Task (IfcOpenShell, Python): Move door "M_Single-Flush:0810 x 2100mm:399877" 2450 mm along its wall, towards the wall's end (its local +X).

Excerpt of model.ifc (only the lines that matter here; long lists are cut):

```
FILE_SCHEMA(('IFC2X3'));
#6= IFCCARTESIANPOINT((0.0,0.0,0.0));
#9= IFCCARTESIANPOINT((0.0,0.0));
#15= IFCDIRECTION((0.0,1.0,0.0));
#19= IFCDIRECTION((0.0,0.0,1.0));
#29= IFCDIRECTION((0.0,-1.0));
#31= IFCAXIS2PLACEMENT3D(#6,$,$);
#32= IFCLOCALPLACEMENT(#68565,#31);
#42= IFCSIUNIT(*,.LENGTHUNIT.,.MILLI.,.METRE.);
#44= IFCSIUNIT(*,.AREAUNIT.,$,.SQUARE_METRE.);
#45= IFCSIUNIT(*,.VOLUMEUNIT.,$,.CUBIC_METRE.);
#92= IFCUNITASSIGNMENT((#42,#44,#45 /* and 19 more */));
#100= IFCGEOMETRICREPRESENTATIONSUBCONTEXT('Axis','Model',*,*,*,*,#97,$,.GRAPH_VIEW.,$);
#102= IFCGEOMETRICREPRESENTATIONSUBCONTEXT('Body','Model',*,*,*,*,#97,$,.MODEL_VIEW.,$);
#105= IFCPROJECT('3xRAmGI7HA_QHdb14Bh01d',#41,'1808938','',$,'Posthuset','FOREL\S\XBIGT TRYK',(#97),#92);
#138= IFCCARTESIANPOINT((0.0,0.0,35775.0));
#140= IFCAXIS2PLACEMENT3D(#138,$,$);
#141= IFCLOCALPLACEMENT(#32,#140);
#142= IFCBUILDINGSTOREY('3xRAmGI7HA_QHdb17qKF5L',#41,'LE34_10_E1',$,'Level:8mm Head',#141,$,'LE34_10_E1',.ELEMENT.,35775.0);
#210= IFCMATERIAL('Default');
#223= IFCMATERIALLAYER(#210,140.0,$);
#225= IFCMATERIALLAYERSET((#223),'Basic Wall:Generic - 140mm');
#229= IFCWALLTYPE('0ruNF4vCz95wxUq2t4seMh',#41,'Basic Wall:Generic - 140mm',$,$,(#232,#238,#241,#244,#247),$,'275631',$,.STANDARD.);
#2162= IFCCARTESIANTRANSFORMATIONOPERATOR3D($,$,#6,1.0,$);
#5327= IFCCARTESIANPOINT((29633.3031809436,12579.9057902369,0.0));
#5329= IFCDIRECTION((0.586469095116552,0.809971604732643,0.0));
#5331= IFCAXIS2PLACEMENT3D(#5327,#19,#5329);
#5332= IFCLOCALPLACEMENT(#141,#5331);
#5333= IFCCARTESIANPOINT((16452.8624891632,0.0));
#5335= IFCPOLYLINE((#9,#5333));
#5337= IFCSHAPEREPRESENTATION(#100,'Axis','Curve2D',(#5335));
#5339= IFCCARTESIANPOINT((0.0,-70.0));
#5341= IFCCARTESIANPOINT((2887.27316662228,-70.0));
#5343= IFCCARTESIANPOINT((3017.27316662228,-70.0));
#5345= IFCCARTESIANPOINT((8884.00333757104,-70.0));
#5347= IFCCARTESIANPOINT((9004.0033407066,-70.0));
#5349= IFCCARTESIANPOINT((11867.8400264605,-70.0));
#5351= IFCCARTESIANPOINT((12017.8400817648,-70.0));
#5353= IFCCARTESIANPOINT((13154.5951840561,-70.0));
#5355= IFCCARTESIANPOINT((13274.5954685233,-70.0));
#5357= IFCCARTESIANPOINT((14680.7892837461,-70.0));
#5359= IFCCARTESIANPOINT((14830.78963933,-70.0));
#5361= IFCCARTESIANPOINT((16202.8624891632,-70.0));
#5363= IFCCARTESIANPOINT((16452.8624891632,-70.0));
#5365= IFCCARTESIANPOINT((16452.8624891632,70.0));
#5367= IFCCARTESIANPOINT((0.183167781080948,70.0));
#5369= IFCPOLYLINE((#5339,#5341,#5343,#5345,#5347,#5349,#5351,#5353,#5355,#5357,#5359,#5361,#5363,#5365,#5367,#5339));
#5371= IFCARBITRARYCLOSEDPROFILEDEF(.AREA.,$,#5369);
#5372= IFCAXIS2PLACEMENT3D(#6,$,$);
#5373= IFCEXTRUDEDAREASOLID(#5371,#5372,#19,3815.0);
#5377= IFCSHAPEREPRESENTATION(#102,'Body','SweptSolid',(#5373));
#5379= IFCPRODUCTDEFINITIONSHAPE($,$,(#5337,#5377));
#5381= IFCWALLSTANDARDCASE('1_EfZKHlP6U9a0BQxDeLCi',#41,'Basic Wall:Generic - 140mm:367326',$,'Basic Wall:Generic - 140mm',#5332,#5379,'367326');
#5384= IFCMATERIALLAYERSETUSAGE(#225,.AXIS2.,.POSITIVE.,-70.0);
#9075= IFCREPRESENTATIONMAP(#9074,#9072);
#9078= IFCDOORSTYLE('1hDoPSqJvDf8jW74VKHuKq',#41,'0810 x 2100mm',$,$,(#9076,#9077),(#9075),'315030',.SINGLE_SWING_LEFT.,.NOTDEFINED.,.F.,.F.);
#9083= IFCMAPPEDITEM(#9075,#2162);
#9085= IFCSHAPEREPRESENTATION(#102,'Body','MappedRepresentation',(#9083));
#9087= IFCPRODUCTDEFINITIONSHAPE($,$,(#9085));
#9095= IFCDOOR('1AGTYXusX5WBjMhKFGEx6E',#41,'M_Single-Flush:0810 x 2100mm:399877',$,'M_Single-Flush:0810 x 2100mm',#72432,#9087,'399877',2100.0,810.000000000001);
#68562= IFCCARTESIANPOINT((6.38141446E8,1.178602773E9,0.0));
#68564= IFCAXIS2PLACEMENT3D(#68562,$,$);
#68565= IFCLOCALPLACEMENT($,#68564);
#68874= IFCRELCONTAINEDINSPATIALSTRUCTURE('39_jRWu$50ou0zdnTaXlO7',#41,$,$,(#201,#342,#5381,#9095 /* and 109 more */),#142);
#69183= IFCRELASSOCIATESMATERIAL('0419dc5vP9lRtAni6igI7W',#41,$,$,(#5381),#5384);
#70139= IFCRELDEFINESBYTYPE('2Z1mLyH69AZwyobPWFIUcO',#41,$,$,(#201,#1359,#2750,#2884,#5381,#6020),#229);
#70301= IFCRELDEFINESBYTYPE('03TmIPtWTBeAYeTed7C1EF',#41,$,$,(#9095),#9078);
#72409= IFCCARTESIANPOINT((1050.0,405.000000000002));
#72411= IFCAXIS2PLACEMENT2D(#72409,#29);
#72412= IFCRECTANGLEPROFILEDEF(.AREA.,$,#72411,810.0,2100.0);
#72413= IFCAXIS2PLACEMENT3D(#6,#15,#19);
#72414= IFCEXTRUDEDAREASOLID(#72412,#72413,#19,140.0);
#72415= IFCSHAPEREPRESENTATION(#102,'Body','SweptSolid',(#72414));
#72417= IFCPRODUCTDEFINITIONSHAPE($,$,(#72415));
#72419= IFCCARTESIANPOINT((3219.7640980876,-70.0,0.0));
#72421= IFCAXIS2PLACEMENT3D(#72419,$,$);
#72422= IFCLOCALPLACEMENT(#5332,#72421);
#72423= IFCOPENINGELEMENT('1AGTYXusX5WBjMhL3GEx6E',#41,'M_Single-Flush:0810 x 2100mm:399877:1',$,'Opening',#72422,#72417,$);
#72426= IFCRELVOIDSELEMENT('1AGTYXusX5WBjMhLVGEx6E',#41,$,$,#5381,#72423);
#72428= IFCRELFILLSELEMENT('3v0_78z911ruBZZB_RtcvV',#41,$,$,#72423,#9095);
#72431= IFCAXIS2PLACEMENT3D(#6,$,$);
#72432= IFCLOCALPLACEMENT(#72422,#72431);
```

```python
import ifcopenshell
import ifcopenshell.api.geometry
import ifcopenshell.util.placement
import ifcopenshell.util.unit

model = ifcopenshell.open("model.ifc")
unit_scale = ifcopenshell.util.unit.calculate_unit_scale(model)

door = model.by_guid("1AGTYXusX5WBjMhKFGEx6E")
opening = door.FillsVoids[0].RelatingOpeningElement
wall = opening.VoidsElements[0].RelatingBuildingElement

wall_matrix = ifcopenshell.util.placement.get_local_placement(wall.ObjectPlacement)
shift = wall_matrix[:3, 0] * 2.45 / unit_scale
before = ifcopenshell.util.placement.get_local_placement(door.ObjectPlacement)[:3, 3].copy()

# The door is placed relative to its opening, so it follows when the opening moves.
matrix = ifcopenshell.util.placement.get_local_placement(opening.ObjectPlacement)
matrix[:3, 3] += shift
ifcopenshell.api.geometry.edit_object_placement(
    model, product=opening, matrix=matrix, is_si=False, should_transform_children=True
)

after = ifcopenshell.util.placement.get_local_placement(door.ObjectPlacement)[:3, 3]
print("door moved by", (after - before).round(3) + 0.0)

model.write("model_edited.ifc")
```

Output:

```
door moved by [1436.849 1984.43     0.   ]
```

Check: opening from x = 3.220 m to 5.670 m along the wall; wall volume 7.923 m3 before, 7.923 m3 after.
